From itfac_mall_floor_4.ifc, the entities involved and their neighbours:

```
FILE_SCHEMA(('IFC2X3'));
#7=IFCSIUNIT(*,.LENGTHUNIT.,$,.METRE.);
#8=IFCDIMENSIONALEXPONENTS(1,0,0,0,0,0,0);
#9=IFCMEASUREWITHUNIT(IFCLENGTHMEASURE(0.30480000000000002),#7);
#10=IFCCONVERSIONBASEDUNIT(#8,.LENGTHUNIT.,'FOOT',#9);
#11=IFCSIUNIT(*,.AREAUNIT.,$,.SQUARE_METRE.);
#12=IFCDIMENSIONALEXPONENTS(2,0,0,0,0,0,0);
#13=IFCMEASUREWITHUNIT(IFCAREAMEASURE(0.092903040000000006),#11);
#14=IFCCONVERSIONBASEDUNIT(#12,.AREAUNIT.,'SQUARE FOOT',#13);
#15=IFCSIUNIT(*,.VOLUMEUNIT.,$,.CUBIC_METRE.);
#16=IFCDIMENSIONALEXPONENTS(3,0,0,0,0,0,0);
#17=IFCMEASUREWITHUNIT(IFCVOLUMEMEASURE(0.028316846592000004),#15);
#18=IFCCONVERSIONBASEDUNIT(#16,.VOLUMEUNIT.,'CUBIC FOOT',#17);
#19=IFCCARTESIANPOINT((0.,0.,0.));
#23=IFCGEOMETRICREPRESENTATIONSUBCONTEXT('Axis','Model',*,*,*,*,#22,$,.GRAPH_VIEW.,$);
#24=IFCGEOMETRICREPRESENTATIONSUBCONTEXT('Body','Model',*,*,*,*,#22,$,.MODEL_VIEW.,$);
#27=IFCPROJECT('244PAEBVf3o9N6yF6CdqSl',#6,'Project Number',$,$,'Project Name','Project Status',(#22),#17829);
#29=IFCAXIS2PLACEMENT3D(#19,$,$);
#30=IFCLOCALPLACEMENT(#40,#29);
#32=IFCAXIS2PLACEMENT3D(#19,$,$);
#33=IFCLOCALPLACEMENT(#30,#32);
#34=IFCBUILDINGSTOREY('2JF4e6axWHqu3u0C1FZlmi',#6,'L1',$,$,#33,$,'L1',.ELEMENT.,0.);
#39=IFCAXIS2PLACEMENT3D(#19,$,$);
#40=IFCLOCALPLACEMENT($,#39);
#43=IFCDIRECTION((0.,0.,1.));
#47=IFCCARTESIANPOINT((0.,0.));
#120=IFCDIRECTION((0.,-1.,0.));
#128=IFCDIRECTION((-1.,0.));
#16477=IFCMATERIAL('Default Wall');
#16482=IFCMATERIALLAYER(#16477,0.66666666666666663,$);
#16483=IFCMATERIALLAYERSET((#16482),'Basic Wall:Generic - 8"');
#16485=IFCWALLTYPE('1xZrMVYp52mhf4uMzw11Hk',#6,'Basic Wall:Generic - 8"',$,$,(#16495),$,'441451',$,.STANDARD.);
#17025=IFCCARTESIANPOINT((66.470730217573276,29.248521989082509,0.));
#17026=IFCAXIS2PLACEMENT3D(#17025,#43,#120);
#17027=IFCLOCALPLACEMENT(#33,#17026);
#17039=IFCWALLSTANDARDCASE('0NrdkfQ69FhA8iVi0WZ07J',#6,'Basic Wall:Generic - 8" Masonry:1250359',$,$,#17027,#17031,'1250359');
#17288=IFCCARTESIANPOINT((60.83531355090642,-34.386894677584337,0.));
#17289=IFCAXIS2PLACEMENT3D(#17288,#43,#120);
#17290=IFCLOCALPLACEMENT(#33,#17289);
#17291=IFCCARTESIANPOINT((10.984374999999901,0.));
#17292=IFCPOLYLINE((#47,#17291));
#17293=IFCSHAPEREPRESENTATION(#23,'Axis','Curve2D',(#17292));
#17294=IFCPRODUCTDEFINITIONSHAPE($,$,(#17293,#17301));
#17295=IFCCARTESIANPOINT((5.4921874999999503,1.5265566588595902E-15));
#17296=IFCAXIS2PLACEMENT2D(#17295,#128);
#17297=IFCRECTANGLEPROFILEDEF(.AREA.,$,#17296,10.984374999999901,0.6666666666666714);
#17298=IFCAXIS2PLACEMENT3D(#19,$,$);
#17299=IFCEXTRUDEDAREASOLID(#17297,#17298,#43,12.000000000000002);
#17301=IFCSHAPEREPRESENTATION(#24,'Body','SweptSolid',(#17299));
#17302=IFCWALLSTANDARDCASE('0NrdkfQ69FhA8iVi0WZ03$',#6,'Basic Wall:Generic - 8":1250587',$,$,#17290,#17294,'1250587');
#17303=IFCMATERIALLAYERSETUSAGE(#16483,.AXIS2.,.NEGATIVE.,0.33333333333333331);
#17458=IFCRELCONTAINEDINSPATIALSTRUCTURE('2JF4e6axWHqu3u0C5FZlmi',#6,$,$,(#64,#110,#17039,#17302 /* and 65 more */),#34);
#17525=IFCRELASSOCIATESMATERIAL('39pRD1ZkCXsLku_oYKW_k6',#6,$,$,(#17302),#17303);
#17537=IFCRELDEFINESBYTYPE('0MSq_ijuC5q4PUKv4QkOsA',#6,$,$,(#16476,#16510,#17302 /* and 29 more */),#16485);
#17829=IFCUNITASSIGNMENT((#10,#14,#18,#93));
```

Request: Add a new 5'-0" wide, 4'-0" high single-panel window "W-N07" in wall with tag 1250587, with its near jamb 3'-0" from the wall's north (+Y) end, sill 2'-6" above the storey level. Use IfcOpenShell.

```python
import numpy as np
import ifcopenshell
import ifcopenshell.api.feature
import ifcopenshell.api.geometry
import ifcopenshell.api.root
import ifcopenshell.api.spatial
import ifcopenshell.api.type
import ifcopenshell.geom
import ifcopenshell.util.element
import ifcopenshell.util.placement
import ifcopenshell.util.representation
import ifcopenshell.util.shape
import ifcopenshell.util.unit

model = ifcopenshell.open("itfac_mall_floor_4.ifc")
unit_scale = ifcopenshell.util.unit.calculate_unit_scale(model)
settings = ifcopenshell.geom.settings()


def volume(element):
    """Net volume in cubic metres, openings subtracted."""
    shape = ifcopenshell.geom.create_shape(settings, element)
    return ifcopenshell.util.shape.get_volume(shape.geometry)


wall = model.by_id(17302)
storey = ifcopenshell.util.element.get_container(wall, ifc_class="IfcBuildingStorey")
context = ifcopenshell.util.representation.get_context(model, "Model", "Body", "MODEL_VIEW")
before = volume(wall)

width, height, from_end, sill = 1.524, 1.2192, 0.9144, 0.762  # metres

# The wall runs along its own X axis, and the end named is its -X end.
wall_shape = ifcopenshell.geom.create_shape(settings, wall)
x, y, z = ifcopenshell.util.shape.get_vertices(wall_shape.geometry).T
start = x.min() + from_end
face, thickness = float(y.min()), float(y.max() - y.min())
wall_matrix = ifcopenshell.util.placement.get_local_placement(wall.ObjectPlacement)
level = ifcopenshell.util.placement.get_local_placement(storey.ObjectPlacement)[2, 3]


def in_wall(x, y):
    """Placement at x, y metres in the wall's axes, at sill height."""
    matrix = wall_matrix.copy()
    matrix[:, 3] = wall_matrix @ np.array([x / unit_scale, y / unit_scale, 0.0, 1.0])
    matrix[2, 3] = level + sill / unit_scale
    return matrix


# Opening: a box that overshoots both wall faces by 50 mm.
opening = ifcopenshell.api.root.create_entity(model, ifc_class="IfcOpeningElement")
box = ifcopenshell.api.geometry.add_wall_representation(
    model, context=context, length=width, height=height, thickness=thickness + 0.1
)
ifcopenshell.api.geometry.assign_representation(model, product=opening, representation=box)
ifcopenshell.api.geometry.edit_object_placement(model, product=opening, matrix=in_wall(start, face - 0.05), is_si=False)
ifcopenshell.api.feature.add_feature(model, feature=opening, element=wall)

window = ifcopenshell.api.root.create_entity(model, ifc_class="IfcWindow", name="W-N07")
window.OverallWidth, window.OverallHeight = width / unit_scale, height / unit_scale
body = ifcopenshell.api.geometry.add_window_representation(
    model,
    context=context,
    overall_width=window.OverallWidth,
    overall_height=window.OverallHeight,
    partition_type="SINGLE_PANEL",
)
ifcopenshell.api.geometry.assign_representation(model, product=window, representation=body)
ifcopenshell.api.spatial.assign_container(model, products=[window], relating_structure=storey)
fills = ifcopenshell.api.feature.add_filling(model, opening=opening, element=window)
fills.OwnerHistory = window.OwnerHistory  # required in IFC2X3

# IFC2X3 keeps the operation on the window style.
style = ifcopenshell.api.root.create_entity(model, ifc_class="IfcWindowStyle", name="W-N07")
style.OperationType, style.ConstructionType = "SINGLE_PANEL", "NOTDEFINED"
style.ParameterTakesPrecedence = style.Sizeable = False
ifcopenshell.api.type.assign_type(model, related_objects=[window], relating_type=style)

# Centre the window in the wall's thickness.
ifcopenshell.api.geometry.edit_object_placement(model, product=window, matrix=in_wall(start, face), is_si=False)
window_shape = ifcopenshell.geom.create_shape(settings, window)
depth = ifcopenshell.util.shape.get_vertices(window_shape.geometry)[:, 1]
offset = face + thickness / 2 - (depth.min() + depth.max()) / 2
ifcopenshell.api.geometry.edit_object_placement(model, product=window, matrix=in_wall(start, offset), is_si=False)

after = volume(wall)

print(f"wall volume {before:.3f} -> {after:.3f} m3")

model.write("itfac_mall_floor_4_updated.ifc")
```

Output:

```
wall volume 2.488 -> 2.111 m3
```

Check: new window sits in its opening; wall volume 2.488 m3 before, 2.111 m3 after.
